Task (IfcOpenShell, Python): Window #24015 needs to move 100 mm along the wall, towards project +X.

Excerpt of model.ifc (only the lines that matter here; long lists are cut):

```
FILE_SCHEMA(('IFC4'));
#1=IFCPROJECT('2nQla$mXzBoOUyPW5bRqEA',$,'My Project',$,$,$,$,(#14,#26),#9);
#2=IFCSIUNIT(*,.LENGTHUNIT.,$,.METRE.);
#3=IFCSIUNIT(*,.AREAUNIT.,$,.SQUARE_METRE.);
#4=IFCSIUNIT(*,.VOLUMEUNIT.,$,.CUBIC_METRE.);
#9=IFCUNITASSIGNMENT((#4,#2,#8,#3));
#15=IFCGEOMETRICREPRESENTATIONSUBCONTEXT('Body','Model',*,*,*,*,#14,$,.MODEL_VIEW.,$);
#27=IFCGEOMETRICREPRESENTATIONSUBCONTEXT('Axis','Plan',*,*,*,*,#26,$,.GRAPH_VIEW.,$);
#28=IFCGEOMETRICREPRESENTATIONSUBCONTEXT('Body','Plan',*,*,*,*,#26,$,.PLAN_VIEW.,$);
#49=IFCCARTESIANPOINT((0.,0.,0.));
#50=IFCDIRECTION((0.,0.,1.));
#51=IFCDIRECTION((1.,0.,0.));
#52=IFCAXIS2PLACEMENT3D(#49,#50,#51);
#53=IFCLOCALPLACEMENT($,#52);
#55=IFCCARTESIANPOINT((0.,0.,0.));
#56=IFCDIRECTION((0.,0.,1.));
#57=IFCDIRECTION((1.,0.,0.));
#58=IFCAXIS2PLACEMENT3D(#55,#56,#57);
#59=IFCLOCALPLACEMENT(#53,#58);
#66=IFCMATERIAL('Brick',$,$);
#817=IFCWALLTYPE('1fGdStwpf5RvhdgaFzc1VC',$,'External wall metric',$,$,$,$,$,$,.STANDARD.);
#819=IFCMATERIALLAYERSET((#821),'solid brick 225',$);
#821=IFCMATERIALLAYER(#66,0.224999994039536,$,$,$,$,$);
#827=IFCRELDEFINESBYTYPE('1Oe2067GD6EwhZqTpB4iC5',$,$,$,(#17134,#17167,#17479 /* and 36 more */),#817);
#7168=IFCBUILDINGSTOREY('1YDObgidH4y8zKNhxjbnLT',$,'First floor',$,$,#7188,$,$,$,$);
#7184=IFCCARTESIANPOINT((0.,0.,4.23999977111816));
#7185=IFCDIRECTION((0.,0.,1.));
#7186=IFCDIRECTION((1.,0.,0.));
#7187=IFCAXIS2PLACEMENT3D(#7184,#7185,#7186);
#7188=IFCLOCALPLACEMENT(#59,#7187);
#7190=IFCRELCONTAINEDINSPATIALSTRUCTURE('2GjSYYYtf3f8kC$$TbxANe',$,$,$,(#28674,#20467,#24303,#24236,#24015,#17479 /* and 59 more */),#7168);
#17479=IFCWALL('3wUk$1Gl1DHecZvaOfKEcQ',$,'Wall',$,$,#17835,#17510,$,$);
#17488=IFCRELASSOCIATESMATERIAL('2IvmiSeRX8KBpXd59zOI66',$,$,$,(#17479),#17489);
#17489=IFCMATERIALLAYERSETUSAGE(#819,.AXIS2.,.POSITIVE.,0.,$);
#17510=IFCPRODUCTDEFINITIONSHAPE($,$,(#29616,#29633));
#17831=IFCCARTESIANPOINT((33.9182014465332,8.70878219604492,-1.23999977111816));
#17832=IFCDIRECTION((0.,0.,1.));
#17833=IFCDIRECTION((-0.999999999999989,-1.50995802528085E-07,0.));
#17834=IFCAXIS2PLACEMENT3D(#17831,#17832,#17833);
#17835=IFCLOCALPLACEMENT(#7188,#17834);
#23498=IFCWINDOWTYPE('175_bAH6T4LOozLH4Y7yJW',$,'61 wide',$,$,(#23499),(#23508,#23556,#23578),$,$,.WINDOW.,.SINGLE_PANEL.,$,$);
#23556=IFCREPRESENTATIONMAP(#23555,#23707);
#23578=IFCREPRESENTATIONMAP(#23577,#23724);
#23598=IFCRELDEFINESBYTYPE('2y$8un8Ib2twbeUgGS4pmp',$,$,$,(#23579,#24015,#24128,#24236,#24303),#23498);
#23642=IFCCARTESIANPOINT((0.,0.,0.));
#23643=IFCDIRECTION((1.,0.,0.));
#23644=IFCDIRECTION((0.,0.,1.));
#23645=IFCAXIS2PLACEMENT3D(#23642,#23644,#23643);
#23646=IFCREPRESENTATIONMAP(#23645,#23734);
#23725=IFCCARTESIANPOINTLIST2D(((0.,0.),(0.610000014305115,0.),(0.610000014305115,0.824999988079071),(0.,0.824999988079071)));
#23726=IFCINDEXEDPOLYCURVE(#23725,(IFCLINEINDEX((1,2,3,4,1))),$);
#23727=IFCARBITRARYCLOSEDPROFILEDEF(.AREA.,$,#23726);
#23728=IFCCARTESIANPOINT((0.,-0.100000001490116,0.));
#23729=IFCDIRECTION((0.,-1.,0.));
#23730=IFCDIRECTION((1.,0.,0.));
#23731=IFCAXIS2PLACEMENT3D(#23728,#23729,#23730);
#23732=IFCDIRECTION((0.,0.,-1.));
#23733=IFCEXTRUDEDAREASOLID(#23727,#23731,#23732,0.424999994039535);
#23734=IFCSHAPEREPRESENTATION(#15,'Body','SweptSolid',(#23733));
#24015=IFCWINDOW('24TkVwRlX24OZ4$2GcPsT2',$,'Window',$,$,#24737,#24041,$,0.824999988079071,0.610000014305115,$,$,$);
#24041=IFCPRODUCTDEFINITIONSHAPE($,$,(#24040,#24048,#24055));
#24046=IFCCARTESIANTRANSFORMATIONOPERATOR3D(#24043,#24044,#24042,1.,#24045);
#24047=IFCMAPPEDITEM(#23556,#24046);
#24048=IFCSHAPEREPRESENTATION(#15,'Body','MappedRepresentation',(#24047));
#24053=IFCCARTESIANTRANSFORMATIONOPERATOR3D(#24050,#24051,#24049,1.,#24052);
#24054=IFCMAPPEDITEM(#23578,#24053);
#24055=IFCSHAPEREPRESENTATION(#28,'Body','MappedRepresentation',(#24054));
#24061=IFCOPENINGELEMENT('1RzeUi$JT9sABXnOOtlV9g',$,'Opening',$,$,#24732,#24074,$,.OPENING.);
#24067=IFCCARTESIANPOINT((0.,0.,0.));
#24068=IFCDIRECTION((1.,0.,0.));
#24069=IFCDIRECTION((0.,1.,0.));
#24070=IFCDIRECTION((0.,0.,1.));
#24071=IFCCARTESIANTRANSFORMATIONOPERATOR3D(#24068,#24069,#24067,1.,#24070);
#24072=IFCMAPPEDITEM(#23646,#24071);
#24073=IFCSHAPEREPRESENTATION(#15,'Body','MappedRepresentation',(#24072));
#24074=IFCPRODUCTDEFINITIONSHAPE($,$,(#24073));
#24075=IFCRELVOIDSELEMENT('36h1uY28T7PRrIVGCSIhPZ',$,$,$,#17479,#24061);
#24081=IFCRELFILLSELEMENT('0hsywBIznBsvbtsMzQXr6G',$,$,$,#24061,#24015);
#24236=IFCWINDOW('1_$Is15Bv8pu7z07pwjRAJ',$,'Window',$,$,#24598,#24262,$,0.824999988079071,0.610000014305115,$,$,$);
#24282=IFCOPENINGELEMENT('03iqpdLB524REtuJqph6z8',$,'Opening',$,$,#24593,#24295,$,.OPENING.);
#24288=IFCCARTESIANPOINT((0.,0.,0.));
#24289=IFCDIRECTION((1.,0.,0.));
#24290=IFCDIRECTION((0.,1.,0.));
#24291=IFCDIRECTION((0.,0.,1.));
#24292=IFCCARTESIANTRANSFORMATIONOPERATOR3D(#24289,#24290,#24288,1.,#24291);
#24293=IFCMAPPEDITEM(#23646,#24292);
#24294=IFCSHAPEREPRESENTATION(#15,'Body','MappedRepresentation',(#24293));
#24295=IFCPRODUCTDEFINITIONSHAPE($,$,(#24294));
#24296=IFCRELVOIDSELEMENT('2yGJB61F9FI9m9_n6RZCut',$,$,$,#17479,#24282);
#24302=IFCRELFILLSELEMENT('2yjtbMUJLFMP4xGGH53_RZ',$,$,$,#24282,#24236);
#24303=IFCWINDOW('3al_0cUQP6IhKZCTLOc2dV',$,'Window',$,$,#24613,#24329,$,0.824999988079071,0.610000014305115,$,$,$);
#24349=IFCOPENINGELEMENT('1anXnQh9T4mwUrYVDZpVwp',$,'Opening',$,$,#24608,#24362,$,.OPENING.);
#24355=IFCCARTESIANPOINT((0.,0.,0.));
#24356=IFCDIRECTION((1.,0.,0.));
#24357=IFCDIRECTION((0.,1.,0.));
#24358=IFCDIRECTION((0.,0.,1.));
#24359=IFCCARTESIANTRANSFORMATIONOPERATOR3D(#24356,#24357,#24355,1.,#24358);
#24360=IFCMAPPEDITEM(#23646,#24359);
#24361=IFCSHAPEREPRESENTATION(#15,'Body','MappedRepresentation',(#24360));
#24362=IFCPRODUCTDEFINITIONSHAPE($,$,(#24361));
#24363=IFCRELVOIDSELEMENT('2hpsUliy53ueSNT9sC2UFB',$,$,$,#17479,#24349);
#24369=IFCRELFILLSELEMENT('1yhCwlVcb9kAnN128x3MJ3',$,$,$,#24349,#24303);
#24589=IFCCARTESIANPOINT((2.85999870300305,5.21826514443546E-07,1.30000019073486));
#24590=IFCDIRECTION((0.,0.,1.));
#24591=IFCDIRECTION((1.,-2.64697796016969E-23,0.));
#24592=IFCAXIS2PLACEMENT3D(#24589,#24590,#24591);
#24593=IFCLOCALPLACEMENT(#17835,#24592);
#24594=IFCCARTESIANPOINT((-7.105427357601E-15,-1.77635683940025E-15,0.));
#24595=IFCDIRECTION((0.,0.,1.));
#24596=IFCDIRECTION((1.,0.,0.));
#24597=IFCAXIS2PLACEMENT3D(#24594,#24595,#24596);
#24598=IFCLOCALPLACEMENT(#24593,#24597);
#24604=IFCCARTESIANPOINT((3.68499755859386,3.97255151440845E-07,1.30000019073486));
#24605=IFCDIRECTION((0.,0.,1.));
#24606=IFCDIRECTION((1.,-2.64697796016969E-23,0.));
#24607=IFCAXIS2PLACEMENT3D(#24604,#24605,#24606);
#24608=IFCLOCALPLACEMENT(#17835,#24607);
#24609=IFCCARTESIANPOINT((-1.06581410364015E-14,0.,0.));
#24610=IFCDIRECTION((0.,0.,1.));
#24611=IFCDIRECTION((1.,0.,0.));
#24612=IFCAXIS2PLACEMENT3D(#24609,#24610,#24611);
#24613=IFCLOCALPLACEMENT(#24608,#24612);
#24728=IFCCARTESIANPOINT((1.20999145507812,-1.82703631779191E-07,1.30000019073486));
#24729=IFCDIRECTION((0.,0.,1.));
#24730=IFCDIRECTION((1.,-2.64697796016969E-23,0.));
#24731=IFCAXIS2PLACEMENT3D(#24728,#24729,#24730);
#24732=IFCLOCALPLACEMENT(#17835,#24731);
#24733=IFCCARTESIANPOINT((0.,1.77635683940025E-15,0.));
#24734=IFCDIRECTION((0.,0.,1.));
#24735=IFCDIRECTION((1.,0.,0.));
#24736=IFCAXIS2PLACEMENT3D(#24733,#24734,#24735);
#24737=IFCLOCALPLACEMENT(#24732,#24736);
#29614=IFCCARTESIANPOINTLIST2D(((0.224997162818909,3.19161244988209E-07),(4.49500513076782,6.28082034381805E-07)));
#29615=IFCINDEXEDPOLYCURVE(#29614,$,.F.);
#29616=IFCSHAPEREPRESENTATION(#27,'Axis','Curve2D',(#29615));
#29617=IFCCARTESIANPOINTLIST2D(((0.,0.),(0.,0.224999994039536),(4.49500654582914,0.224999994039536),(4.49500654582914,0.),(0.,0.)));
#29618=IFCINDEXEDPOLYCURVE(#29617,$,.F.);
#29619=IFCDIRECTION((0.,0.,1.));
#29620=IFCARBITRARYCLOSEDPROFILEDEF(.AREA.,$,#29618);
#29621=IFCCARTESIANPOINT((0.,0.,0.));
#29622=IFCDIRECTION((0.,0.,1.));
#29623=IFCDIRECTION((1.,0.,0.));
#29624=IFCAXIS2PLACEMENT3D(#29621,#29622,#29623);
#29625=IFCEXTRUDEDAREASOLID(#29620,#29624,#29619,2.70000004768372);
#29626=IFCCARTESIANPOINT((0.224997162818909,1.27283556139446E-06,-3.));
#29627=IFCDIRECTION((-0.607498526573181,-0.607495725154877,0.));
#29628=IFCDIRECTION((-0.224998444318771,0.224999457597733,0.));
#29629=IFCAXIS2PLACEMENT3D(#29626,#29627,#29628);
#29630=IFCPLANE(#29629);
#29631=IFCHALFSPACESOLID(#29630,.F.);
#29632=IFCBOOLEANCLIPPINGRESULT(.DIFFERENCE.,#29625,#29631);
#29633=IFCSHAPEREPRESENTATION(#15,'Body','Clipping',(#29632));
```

```python
import ifcopenshell
import ifcopenshell.api.geometry
import ifcopenshell.util.placement

model = ifcopenshell.open("model.ifc")

window = model.by_id(24015)
opening = window.FillsVoids[0].RelatingOpeningElement
wall = opening.VoidsElements[0].RelatingBuildingElement

wall_matrix = ifcopenshell.util.placement.get_local_placement(wall.ObjectPlacement)
shift = wall_matrix[:3, 0] * -0.1
before = ifcopenshell.util.placement.get_local_placement(window.ObjectPlacement)[:3, 3].copy()

# The window is placed relative to its opening, so it follows when the opening moves.
matrix = ifcopenshell.util.placement.get_local_placement(opening.ObjectPlacement)
matrix[:3, 3] += shift
ifcopenshell.api.geometry.edit_object_placement(
    model, product=opening, matrix=matrix, is_si=False, should_transform_children=True
)

after = ifcopenshell.util.placement.get_local_placement(window.ObjectPlacement)[:3, 3]
print("window moved by", (after - before).round(3) + 0.0)

model.write("model_edited.ifc")
```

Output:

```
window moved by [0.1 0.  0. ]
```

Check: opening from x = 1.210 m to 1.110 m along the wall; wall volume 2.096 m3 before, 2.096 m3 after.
